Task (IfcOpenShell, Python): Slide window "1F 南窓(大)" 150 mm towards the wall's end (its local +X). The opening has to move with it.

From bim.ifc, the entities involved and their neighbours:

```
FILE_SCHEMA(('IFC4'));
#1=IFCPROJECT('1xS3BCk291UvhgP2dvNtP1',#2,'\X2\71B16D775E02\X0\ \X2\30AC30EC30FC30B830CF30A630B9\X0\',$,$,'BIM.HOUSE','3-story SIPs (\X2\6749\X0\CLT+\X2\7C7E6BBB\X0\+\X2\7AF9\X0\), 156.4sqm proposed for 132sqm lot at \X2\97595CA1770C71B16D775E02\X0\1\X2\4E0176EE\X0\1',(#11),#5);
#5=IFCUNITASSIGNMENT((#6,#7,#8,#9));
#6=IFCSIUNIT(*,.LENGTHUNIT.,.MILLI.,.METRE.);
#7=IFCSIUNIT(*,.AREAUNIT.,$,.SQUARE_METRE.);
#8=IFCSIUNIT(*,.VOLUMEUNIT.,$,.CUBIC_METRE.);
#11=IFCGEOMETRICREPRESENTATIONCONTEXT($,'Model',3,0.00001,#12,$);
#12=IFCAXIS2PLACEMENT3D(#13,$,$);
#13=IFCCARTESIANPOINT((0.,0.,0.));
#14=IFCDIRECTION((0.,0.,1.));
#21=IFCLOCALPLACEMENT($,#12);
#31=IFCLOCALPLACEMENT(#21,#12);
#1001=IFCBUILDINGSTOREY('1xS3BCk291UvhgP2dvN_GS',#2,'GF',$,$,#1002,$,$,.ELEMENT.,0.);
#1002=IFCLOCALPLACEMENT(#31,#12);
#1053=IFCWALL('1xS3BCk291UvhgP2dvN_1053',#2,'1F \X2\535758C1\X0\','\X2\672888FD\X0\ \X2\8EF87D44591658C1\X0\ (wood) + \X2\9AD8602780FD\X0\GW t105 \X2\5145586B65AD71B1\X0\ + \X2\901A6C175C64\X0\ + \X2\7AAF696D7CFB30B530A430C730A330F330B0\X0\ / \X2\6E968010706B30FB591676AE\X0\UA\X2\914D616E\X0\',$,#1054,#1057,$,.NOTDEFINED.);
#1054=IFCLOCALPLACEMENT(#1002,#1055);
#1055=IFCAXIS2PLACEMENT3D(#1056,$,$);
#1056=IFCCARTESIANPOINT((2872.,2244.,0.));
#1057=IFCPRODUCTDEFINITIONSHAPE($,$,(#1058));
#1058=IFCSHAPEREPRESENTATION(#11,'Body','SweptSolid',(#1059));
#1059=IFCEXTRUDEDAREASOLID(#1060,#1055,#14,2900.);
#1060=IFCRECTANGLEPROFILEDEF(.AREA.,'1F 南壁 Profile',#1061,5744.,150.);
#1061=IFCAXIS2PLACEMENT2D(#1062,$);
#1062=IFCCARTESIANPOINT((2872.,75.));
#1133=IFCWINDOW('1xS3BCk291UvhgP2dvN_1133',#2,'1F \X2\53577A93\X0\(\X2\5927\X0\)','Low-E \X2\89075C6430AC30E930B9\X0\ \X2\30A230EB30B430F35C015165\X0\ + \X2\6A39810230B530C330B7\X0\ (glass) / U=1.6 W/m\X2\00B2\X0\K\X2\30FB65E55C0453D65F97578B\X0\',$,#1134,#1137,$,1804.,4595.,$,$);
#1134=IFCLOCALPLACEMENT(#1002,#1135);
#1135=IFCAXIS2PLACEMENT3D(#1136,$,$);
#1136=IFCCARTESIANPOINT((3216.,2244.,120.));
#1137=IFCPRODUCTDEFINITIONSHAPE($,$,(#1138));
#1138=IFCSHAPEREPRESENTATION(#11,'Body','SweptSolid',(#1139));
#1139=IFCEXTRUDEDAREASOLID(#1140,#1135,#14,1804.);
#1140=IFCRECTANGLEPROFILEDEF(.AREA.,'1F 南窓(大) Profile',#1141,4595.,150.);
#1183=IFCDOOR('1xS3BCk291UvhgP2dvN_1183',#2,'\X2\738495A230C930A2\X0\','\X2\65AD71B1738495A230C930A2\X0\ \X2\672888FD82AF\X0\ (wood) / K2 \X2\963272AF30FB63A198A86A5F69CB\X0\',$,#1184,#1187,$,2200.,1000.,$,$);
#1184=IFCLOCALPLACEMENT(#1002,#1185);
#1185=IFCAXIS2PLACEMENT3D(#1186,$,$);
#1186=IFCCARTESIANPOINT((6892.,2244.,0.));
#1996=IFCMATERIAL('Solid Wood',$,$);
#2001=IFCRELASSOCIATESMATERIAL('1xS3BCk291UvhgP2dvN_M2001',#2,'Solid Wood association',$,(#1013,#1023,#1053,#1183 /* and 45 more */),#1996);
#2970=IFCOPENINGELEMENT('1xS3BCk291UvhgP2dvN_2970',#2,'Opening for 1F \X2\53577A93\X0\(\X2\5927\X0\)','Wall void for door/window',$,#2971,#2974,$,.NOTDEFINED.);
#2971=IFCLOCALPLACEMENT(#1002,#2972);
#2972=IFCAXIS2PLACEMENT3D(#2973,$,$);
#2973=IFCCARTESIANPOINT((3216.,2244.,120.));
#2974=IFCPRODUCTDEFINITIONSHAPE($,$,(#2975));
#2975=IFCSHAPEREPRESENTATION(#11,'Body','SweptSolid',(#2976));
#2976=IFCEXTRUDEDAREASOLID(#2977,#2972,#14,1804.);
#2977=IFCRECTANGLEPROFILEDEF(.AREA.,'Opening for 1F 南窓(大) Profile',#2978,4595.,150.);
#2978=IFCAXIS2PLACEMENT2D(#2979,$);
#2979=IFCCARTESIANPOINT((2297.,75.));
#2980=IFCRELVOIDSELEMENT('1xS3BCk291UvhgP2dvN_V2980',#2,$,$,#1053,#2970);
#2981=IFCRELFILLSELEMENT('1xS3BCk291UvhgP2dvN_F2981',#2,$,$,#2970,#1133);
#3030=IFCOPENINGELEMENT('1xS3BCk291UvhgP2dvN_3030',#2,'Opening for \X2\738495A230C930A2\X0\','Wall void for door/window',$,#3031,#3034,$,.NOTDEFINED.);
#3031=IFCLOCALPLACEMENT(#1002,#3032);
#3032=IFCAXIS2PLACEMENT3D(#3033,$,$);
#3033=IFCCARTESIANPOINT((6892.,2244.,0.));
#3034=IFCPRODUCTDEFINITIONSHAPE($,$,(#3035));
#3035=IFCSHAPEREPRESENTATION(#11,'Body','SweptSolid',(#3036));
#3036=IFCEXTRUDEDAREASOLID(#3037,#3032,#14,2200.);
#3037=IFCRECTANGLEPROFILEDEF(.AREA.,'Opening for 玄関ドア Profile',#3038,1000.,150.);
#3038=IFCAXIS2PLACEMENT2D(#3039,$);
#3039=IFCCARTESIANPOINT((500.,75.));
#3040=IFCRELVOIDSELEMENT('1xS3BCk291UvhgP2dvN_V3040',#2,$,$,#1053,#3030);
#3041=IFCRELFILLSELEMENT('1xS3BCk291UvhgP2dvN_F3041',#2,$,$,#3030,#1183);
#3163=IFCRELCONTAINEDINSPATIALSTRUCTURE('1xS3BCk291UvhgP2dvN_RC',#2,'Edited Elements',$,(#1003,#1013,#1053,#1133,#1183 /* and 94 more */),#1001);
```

```python
import ifcopenshell
import ifcopenshell.api.geometry
import ifcopenshell.util.placement
import ifcopenshell.util.unit

model = ifcopenshell.open("bim.ifc")
unit_scale = ifcopenshell.util.unit.calculate_unit_scale(model)

window = model.by_guid("1xS3BCk291UvhgP2dvN_1133")
opening = window.FillsVoids[0].RelatingOpeningElement
wall = opening.VoidsElements[0].RelatingBuildingElement

wall_matrix = ifcopenshell.util.placement.get_local_placement(wall.ObjectPlacement)
shift = wall_matrix[:3, 0] * 0.15 / unit_scale
before = ifcopenshell.util.placement.get_local_placement(window.ObjectPlacement)[:3, 3].copy()

# The window is not placed relative to its opening, so move both.
for product in (opening, window):
    matrix = ifcopenshell.util.placement.get_local_placement(product.ObjectPlacement)
    matrix[:3, 3] += shift
    ifcopenshell.api.geometry.edit_object_placement(model, product=product, matrix=matrix, is_si=False)

after = ifcopenshell.util.placement.get_local_placement(window.ObjectPlacement)[:3, 3]
print("window moved by", (after - before).round(3) + 0.0)

model.write("bim_updated.ifc")
```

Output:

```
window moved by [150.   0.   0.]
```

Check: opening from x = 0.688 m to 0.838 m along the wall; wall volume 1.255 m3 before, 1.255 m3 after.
